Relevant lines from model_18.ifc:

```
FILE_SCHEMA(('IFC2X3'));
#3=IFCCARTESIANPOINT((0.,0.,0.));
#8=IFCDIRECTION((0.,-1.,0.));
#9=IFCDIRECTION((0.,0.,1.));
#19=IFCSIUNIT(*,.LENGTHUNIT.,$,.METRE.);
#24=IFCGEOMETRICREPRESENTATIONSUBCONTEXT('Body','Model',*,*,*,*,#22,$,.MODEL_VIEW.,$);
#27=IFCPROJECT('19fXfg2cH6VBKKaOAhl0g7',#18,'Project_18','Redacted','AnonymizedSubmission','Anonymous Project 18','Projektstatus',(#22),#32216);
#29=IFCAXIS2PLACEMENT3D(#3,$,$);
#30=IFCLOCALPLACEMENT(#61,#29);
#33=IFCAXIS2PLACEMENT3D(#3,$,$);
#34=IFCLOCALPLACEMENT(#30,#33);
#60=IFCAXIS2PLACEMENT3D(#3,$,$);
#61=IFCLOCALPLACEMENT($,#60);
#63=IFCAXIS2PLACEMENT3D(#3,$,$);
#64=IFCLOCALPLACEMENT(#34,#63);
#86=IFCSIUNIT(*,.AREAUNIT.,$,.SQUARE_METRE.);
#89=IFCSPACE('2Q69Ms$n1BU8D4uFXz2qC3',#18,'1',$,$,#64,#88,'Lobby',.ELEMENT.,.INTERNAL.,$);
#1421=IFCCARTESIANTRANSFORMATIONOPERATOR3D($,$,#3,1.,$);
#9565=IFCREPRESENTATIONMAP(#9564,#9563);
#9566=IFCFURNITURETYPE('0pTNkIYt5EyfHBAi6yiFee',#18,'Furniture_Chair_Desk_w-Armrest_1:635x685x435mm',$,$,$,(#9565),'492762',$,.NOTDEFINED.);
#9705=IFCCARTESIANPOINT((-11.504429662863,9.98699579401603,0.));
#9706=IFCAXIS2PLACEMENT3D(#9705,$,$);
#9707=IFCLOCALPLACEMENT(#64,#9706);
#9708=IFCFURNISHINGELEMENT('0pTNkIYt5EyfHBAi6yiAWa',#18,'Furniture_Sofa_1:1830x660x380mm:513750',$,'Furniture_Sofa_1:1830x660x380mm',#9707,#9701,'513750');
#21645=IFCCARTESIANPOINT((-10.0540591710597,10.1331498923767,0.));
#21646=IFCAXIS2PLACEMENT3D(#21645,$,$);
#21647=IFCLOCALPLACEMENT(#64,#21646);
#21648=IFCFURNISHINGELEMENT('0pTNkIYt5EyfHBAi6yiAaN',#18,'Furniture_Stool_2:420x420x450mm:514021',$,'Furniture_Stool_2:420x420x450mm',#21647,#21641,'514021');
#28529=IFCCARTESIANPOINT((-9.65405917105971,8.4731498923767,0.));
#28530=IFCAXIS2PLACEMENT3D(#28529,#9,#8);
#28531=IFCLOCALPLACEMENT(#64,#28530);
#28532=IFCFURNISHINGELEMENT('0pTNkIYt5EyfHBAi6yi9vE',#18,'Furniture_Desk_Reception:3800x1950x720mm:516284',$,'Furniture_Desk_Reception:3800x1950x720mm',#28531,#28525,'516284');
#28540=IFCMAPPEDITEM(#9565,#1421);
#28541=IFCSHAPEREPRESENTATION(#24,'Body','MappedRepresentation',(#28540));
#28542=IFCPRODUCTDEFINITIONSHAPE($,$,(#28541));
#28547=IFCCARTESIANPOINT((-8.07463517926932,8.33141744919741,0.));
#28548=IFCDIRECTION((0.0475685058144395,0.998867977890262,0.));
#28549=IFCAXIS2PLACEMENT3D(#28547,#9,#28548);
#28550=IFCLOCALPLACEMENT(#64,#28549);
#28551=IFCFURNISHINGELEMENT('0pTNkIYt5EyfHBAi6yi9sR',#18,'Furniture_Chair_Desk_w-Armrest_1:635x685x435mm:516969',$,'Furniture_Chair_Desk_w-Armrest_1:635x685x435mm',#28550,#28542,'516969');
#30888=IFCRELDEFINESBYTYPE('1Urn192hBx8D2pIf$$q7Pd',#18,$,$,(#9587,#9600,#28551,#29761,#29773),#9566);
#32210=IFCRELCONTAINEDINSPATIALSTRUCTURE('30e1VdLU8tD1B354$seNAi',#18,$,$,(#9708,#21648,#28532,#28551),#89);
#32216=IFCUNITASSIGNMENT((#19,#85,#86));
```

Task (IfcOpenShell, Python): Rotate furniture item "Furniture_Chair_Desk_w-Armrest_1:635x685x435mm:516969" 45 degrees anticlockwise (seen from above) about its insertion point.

```python
import ifcopenshell
import ifcopenshell.api.geometry
import ifcopenshell.util.placement

model = ifcopenshell.open("model_18.ifc")

item = model.by_guid("0pTNkIYt5EyfHBAi6yi9sR")
matrix = ifcopenshell.util.placement.get_local_placement(item.ObjectPlacement)
matrix = matrix @ ifcopenshell.util.placement.rotation(45, "Z")
ifcopenshell.api.geometry.edit_object_placement(model, product=item, matrix=matrix, is_si=False)

print(ifcopenshell.util.placement.get_local_placement(item.ObjectPlacement).round(3) + 0.0)

model.write("model_18_edited.ifc")
```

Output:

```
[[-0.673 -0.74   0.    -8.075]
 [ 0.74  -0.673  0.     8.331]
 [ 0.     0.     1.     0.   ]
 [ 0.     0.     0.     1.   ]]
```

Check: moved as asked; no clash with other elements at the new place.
